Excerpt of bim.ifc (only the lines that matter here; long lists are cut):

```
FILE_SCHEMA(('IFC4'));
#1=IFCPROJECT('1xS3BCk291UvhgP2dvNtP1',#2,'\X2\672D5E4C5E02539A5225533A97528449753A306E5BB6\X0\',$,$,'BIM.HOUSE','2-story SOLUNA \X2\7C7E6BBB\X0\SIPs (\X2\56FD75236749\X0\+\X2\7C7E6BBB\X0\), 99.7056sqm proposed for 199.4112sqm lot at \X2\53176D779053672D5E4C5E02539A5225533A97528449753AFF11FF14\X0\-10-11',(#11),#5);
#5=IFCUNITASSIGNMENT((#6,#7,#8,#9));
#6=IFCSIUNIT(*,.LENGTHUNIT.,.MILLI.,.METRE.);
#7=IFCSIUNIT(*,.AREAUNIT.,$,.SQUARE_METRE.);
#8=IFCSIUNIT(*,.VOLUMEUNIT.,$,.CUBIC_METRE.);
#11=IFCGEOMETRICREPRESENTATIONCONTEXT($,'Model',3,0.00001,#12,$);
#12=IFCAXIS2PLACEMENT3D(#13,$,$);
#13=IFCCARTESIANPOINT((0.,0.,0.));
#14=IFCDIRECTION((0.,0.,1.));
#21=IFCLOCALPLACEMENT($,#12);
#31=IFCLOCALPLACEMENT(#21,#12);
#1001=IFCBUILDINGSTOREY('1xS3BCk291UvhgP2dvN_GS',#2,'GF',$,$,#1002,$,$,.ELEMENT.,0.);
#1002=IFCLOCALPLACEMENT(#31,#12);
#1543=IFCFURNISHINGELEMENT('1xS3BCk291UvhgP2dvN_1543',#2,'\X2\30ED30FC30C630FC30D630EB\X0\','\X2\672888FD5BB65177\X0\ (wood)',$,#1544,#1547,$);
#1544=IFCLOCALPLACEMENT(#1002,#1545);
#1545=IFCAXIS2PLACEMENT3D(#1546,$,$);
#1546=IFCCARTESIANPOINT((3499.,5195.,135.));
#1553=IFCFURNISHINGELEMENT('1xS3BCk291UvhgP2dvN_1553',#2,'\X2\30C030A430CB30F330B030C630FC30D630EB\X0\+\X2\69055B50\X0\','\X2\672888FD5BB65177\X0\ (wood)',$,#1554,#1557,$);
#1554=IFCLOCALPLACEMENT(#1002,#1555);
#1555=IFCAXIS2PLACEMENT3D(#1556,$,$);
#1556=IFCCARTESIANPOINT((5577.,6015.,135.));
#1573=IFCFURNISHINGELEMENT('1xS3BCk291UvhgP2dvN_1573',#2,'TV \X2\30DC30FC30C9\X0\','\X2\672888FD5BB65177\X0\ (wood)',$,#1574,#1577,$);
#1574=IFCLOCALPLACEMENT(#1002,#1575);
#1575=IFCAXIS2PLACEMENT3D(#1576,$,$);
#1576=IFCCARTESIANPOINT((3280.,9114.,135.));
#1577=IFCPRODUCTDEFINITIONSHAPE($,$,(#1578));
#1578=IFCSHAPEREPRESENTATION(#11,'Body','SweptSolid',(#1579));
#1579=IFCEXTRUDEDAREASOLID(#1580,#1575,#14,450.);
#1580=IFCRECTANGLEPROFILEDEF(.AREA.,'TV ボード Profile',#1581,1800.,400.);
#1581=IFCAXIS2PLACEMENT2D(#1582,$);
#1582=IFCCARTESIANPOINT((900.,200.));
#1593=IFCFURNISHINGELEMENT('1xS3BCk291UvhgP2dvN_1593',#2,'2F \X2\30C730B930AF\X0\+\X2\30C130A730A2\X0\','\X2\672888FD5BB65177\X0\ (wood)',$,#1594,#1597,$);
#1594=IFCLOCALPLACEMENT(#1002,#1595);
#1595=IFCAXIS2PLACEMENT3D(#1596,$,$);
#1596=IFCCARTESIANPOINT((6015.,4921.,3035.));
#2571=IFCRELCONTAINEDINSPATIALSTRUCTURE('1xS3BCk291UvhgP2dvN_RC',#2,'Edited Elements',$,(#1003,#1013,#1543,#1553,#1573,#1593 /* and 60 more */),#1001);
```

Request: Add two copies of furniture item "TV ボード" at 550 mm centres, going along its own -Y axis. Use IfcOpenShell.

```python
import ifcopenshell
import ifcopenshell.api.geometry
import ifcopenshell.api.root
import ifcopenshell.util.element
import ifcopenshell.util.placement
import ifcopenshell.util.unit

model = ifcopenshell.open("bim.ifc")
unit_scale = ifcopenshell.util.unit.calculate_unit_scale(model)


def reuse_history(source, copy):
    """copy_class also copies each property set's owner history, people and application; keep the originals."""
    for rel in copy.IsDefinedBy:
        if rel.is_a("IfcRelDefinesByProperties") and (history := rel.RelatingPropertyDefinition.OwnerHistory):
            rel.RelatingPropertyDefinition.OwnerHistory = source.OwnerHistory
            ifcopenshell.util.element.remove_deep2(model, history)


source = model.by_id(1573)
base = ifcopenshell.util.placement.get_local_placement(source.ObjectPlacement)
step = -base[:3, 1] * 0.55 / unit_scale

for i in range(1, 3):
    copy = ifcopenshell.api.root.copy_class(model, product=source)
    copy.Representation = ifcopenshell.util.element.copy_deep(
        model, source.Representation, exclude=["IfcGeometricRepresentationContext", "IfcRepresentationMap"]
    )
    reuse_history(source, copy)
    matrix = base.copy()
    matrix[:3, 3] += i * step
    print("added at", matrix[:3, 3].round(3) + 0.0)
    ifcopenshell.api.geometry.edit_object_placement(model, product=copy, matrix=matrix, is_si=False)

model.write("bim_rev.ifc")
```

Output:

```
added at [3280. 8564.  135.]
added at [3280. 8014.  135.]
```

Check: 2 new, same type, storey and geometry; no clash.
